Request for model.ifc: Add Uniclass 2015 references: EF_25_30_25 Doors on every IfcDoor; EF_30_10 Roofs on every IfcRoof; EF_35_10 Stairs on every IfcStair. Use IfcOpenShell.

First a look at what the model holds.

```python
import ifcopenshell

model = ifcopenshell.open("model.ifc")
print(model.schema)
print("classifications:", [c.Name for c in model.by_type("IfcClassification")])
for ifc_class in ("IfcDoor", "IfcRoof", "IfcStair", "IfcWall", "IfcWindow"):
    print(ifc_class, len(model.by_type(ifc_class)))
```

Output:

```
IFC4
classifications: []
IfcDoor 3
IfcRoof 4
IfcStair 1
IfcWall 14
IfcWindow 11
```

```python
import ifcopenshell
import ifcopenshell.api.classification

model = ifcopenshell.open("model.ifc")

system = ifcopenshell.api.classification.add_classification(model, classification="Uniclass 2015")

codes = {
    "IfcDoor": ("EF_25_30_25", "Doors"),
    "IfcRoof": ("EF_30_10", "Roofs"),
    "IfcStair": ("EF_35_10", "Stairs"),
}
for ifc_class, (code, name) in codes.items():
    products = model.by_type(ifc_class)
    ifcopenshell.api.classification.add_reference(
        model, products=products, classification=system, identification=code, name=name
    )
    print(code, len(products))

model.write("model_edited.ifc")
```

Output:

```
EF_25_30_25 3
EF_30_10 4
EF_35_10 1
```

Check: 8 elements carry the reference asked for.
